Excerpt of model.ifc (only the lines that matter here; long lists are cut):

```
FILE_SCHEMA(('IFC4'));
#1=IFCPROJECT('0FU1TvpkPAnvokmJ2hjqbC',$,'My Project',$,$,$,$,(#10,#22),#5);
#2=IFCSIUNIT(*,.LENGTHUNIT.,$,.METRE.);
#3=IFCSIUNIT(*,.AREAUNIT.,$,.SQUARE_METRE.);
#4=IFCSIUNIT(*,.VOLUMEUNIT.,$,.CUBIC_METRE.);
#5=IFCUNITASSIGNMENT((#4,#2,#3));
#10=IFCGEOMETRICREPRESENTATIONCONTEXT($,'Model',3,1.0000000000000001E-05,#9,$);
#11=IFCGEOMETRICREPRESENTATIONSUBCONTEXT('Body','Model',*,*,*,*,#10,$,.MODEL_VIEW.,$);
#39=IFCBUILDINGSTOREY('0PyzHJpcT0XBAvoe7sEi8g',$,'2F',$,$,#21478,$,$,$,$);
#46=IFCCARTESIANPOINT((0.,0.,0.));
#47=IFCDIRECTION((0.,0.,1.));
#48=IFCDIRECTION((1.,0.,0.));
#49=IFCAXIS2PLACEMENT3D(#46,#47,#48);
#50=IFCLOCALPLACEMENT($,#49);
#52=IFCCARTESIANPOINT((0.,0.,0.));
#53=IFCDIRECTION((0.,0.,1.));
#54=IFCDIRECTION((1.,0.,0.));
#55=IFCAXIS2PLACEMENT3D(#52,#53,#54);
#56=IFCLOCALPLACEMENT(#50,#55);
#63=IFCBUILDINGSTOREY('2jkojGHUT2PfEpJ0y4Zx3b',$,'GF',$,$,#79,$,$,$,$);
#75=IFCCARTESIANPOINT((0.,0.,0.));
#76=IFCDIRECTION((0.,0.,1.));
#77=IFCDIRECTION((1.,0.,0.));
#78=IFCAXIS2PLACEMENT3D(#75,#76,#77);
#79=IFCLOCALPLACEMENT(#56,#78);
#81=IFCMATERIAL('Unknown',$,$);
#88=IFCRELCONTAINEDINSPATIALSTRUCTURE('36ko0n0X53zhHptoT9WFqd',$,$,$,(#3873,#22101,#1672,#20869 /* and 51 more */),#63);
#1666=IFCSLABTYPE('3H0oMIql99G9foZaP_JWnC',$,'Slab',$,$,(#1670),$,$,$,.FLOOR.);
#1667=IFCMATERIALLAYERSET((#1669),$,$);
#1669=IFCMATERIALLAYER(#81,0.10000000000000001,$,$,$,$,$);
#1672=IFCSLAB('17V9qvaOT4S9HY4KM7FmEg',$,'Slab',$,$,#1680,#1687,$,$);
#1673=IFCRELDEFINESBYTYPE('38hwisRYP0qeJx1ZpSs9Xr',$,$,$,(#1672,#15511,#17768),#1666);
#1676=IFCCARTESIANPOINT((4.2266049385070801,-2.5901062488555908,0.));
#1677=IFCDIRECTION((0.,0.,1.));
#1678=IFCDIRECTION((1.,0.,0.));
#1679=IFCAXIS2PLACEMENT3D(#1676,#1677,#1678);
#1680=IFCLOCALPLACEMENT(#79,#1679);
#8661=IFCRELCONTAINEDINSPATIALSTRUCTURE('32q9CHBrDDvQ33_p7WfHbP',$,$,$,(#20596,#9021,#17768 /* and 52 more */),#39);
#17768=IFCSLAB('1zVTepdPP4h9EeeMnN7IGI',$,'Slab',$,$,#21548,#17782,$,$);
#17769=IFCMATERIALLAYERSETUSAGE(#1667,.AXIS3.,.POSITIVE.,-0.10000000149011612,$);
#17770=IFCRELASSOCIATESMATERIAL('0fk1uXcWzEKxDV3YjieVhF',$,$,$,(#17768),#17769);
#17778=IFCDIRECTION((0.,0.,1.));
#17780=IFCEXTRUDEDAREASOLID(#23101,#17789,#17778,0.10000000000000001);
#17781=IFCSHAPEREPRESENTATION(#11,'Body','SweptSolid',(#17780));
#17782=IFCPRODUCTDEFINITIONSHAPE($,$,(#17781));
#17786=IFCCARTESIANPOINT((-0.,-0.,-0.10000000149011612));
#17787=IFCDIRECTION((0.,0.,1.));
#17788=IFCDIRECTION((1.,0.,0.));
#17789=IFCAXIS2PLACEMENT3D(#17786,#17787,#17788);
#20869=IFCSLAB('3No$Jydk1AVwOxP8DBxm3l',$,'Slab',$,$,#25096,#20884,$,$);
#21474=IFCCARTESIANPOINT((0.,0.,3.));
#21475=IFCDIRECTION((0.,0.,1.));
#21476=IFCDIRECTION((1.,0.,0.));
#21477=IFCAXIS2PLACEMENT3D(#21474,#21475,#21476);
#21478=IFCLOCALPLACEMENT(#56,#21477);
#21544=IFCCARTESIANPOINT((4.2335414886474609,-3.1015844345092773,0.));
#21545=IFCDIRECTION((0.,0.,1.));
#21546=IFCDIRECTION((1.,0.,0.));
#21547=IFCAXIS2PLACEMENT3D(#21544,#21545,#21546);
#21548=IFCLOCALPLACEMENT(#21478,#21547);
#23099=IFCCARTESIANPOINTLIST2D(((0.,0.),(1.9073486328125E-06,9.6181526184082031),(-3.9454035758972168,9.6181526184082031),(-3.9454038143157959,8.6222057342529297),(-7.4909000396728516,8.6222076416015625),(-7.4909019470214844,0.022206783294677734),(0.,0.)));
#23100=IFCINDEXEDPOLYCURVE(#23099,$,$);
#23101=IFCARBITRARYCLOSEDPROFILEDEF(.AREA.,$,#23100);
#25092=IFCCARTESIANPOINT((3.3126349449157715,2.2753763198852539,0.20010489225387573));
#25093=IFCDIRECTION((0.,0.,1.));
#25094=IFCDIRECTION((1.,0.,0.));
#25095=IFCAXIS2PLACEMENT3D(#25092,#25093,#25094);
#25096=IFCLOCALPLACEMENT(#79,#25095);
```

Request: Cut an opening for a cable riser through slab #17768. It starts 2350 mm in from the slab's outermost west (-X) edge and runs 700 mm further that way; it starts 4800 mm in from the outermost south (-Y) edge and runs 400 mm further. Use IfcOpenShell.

```python
import numpy as np
import ifcopenshell
import ifcopenshell.api.feature
import ifcopenshell.api.geometry
import ifcopenshell.api.root
import ifcopenshell.geom
import ifcopenshell.util.placement
import ifcopenshell.util.representation
import ifcopenshell.util.shape
import ifcopenshell.util.unit

model = ifcopenshell.open("model.ifc")
unit_scale = ifcopenshell.util.unit.calculate_unit_scale(model)
settings = ifcopenshell.geom.settings()


def volume(element):
    """Net volume in cubic metres, openings subtracted."""
    shape = ifcopenshell.geom.create_shape(settings, element)
    return ifcopenshell.util.shape.get_volume(shape.geometry)


slab = model.by_guid("1zVTepdPP4h9EeeMnN7IGI")
before = volume(slab)

# Extent in the slab's own axes, in metres. The edges named are its -X and -Y sides.
slab_shape = ifcopenshell.geom.create_shape(settings, slab)
vertices = ifcopenshell.util.shape.get_vertices(slab_shape.geometry)
x_min, y_min, bottom = vertices.min(axis=0)
top = vertices[:, 2].max()

opening = ifcopenshell.api.root.create_entity(model, ifc_class="IfcOpeningElement", name="Cable riser opening", predefined_type="OPENING")
context = ifcopenshell.util.representation.get_context(model, "Model", "Body", "MODEL_VIEW")
width, depth = 0.7, 0.4
outline = [(0.0, 0.0), (width, 0.0), (width, depth), (0.0, depth), (0.0, 0.0)]
# Overshoot both faces by 50 mm so the cut is clean.
shape = ifcopenshell.api.geometry.add_slab_representation(
    model, context=context, depth=top - bottom + 0.1, polyline=outline
)
ifcopenshell.api.geometry.assign_representation(model, product=opening, representation=shape)

matrix = ifcopenshell.util.placement.get_local_placement(slab.ObjectPlacement)
matrix[:, 3] = matrix @ np.append(np.array([x_min + 2.35, y_min + 4.8, bottom - 0.05]) / unit_scale, 1.0)
ifcopenshell.api.geometry.edit_object_placement(model, product=opening, matrix=matrix, is_si=False)
ifcopenshell.api.feature.add_feature(model, feature=opening, element=slab)

after = volume(slab)

print(f"slab volume {before:.3f} -> {after:.3f} m3")

model.write("model_v2.ifc")
```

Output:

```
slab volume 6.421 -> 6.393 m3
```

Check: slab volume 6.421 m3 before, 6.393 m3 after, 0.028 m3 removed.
